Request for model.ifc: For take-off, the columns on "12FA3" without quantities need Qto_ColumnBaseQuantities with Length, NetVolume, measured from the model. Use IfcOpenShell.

First a look at what the model holds.

```python
import ifcopenshell
import ifcopenshell.util.element
import ifcopenshell.util.unit

model = ifcopenshell.open("model.ifc")
print(model.schema)
for unit_type in ("LENGTHUNIT", "AREAUNIT", "VOLUMEUNIT"):
    print(unit_type, ifcopenshell.util.unit.calculate_unit_scale(model, unit_type))
storey = next(s for s in model.by_type("IfcBuildingStorey") if s.Name == "12FA3")
columns = [e for e in ifcopenshell.util.element.get_decomposition(storey) if e.is_a("IfcColumn")]
for e in sorted(columns, key=lambda e: e.id()):
    print(e.id(), e.is_a(), e.Name, list(ifcopenshell.util.element.get_psets(e, qtos_only=True)), sep=" | ")
```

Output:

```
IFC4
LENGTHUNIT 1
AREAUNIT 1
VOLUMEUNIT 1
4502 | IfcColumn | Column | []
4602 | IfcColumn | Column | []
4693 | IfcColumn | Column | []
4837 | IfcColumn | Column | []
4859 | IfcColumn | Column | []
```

```python
import ifcopenshell
import ifcopenshell.api.pset
import ifcopenshell.geom
import ifcopenshell.util.element
import ifcopenshell.util.shape
import ifcopenshell.util.unit

model = ifcopenshell.open("model.ifc")
unit_scale = ifcopenshell.util.unit.calculate_unit_scale(model)
volume_scale = ifcopenshell.util.unit.calculate_unit_scale(model, "VOLUMEUNIT")
settings = ifcopenshell.geom.settings()

storey = next(s for s in model.by_type("IfcBuildingStorey") if s.Name == "12FA3")
columns = [e for e in ifcopenshell.util.element.get_decomposition(storey) if e.is_a("IfcColumn")]

for e in sorted(columns, key=lambda e: e.id()):
    if ifcopenshell.util.element.get_psets(e, qtos_only=True, should_inherit=False):
        continue
    # Geometry comes back in metres, in the element's own axes.
    shape = ifcopenshell.geom.create_shape(settings, e)
    values = {
        "Length": ifcopenshell.util.shape.get_z(shape.geometry) / unit_scale,
        "NetVolume": ifcopenshell.util.shape.get_volume(shape.geometry) / volume_scale,
    }
    qto = ifcopenshell.api.pset.add_qto(model, product=e, name="Qto_ColumnBaseQuantities")
    ifcopenshell.api.pset.edit_qto(model, qto=qto, properties=values)
    print(e.id(), {k: round(v, 3) for k, v in values.items()})

model.write("model_updated.ifc")
```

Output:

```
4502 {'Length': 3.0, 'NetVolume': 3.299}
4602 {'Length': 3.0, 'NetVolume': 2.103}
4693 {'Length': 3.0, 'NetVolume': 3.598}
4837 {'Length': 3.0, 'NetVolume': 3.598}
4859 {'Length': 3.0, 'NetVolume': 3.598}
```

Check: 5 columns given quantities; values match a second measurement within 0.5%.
